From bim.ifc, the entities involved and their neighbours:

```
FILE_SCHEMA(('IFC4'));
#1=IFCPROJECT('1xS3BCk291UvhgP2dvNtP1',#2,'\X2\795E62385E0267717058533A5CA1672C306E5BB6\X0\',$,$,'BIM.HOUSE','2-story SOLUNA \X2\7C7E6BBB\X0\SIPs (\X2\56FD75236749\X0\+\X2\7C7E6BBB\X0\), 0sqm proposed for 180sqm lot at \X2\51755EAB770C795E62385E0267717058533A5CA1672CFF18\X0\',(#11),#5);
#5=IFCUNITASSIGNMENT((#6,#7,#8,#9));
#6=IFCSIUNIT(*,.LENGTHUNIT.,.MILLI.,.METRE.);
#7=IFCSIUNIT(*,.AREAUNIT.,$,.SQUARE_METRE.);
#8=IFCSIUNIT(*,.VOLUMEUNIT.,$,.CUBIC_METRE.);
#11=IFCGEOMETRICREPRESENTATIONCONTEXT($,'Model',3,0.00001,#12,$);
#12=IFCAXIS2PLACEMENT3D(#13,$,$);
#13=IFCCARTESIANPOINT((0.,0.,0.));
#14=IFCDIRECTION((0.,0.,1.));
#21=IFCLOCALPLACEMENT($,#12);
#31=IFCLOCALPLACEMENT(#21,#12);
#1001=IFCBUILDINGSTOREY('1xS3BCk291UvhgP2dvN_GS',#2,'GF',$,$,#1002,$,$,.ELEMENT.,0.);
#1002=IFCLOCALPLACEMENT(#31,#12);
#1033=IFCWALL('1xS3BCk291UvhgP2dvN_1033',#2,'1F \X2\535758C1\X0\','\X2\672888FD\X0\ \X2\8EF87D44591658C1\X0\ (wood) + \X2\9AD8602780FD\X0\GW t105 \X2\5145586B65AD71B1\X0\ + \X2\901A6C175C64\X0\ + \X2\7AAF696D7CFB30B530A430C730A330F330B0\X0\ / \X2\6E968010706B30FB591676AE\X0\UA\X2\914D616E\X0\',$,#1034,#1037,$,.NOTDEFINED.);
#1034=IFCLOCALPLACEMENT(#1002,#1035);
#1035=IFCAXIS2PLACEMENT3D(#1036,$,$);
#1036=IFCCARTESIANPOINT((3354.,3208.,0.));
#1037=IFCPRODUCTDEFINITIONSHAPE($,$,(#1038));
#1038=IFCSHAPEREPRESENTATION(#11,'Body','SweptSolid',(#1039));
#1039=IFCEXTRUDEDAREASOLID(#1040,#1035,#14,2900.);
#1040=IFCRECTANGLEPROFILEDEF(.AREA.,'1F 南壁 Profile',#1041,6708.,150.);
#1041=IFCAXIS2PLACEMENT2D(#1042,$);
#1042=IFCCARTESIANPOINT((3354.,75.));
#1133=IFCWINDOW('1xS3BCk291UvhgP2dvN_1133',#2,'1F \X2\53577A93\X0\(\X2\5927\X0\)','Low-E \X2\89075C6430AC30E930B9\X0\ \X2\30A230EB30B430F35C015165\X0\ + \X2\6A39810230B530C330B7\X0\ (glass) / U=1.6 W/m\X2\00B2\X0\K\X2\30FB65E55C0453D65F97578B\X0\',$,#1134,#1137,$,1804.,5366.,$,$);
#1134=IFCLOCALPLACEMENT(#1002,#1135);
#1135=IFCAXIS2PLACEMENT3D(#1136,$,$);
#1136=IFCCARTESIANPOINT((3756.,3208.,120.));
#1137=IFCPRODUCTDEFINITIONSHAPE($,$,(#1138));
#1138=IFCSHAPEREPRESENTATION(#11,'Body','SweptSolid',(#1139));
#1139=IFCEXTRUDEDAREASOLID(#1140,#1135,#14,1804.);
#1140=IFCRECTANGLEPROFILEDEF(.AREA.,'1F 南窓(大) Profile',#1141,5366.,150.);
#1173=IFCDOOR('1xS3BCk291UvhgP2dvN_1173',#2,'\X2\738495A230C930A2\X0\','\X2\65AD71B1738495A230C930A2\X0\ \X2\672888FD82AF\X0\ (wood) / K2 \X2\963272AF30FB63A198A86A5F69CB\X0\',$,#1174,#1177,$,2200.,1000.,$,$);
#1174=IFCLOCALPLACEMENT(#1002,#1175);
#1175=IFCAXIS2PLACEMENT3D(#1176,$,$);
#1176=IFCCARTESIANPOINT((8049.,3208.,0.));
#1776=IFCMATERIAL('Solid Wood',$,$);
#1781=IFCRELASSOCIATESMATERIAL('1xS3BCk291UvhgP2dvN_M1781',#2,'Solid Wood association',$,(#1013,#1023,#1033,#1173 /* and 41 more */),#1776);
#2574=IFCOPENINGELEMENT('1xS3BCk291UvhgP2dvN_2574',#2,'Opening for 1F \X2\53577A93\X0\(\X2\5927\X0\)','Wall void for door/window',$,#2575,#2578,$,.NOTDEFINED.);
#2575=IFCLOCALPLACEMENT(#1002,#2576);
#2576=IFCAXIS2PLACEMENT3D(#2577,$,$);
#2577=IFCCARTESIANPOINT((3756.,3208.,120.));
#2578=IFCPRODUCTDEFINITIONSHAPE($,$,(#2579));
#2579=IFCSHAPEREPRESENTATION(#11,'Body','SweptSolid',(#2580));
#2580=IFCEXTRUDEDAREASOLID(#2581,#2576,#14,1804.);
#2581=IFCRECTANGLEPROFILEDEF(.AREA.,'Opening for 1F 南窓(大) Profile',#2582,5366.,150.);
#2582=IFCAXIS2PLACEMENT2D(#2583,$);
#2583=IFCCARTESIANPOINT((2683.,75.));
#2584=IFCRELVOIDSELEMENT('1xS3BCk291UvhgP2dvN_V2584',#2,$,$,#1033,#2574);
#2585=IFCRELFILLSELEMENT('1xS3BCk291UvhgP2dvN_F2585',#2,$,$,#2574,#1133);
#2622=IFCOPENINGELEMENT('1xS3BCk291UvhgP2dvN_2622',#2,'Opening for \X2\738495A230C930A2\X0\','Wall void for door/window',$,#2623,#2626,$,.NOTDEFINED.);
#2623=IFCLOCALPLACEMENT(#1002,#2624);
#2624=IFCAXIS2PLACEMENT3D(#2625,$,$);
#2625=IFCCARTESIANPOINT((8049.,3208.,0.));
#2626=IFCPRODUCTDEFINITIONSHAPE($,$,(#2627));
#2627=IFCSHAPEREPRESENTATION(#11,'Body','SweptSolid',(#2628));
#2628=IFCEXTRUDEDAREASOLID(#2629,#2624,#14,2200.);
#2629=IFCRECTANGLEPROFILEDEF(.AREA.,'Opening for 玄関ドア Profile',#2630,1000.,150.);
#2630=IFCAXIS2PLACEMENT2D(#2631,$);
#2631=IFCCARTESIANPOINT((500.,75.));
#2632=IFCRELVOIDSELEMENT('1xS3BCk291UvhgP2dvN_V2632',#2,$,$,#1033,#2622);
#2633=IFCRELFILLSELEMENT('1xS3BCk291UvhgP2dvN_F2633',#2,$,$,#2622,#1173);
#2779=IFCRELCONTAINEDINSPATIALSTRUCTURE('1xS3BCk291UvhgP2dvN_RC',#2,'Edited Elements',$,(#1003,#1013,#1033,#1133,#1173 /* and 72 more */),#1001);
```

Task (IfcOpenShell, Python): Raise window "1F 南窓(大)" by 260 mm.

```python
import numpy as np
import ifcopenshell
import ifcopenshell.api.geometry
import ifcopenshell.util.placement
import ifcopenshell.util.unit

model = ifcopenshell.open("bim.ifc")
unit_scale = ifcopenshell.util.unit.calculate_unit_scale(model)

window = model.by_guid("1xS3BCk291UvhgP2dvN_1133")
opening = window.FillsVoids[0].RelatingOpeningElement
dz = 0.26 / unit_scale

shift = np.array([0.0, 0.0, dz])
# The window is not placed relative to its opening, so move both.
for product in (opening, window):
    matrix = ifcopenshell.util.placement.get_local_placement(product.ObjectPlacement)
    matrix[:3, 3] += shift
    ifcopenshell.api.geometry.edit_object_placement(model, product=product, matrix=matrix, is_si=False)

print(f"moved by {dz * unit_scale:+.3f} m")

model.write("bim_rev.ifc")
```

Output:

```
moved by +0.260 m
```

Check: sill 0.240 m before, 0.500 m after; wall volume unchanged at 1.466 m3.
